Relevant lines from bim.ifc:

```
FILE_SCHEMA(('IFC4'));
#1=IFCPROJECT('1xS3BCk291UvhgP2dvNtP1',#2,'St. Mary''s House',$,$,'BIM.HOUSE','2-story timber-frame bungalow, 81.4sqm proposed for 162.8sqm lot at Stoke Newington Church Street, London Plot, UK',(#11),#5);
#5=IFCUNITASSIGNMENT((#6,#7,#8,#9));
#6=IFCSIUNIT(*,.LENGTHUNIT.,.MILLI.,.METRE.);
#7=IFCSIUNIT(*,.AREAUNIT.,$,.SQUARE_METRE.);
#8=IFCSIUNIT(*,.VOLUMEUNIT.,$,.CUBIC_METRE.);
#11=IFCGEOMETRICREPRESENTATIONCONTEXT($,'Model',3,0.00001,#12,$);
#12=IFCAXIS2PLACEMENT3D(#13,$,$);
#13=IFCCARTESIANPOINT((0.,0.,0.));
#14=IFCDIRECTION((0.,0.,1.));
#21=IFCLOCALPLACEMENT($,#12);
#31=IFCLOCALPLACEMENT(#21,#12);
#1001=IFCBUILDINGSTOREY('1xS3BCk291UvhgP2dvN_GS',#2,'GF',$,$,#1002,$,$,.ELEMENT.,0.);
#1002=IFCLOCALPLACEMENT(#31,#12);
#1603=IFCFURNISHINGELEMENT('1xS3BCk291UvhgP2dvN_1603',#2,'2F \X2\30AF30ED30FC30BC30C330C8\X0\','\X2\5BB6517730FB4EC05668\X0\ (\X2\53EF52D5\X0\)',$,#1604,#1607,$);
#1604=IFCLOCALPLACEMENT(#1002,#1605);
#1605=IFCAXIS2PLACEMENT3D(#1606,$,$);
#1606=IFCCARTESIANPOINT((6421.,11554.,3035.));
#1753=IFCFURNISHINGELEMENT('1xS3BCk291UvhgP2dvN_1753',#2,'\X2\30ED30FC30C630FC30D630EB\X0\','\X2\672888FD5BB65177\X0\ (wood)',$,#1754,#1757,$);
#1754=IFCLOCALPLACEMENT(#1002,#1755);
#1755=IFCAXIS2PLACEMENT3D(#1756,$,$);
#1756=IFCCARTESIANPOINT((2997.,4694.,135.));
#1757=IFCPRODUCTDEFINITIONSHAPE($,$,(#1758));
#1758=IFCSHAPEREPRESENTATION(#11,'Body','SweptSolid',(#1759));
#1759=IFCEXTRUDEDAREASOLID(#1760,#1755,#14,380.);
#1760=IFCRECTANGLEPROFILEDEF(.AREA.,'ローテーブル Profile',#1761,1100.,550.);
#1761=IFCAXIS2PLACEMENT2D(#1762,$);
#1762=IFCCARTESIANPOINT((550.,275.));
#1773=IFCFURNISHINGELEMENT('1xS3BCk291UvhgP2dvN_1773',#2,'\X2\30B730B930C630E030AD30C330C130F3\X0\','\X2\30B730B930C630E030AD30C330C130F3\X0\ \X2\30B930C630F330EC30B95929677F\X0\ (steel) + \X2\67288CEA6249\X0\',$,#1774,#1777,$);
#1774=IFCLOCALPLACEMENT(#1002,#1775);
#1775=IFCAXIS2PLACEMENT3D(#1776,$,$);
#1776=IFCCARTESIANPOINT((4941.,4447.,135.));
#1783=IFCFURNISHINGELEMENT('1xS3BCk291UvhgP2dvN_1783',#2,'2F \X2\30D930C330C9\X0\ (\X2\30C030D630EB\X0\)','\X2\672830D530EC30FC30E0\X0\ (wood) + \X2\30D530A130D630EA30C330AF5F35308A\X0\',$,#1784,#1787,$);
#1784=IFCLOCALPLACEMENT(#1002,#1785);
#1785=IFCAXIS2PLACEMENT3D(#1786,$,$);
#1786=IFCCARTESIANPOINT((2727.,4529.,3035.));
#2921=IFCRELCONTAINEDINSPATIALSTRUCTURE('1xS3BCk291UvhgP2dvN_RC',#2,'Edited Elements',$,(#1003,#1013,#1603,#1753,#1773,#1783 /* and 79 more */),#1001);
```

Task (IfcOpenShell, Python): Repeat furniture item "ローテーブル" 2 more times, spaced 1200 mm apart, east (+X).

```python
import numpy as np
import ifcopenshell
import ifcopenshell.api.geometry
import ifcopenshell.api.root
import ifcopenshell.util.element
import ifcopenshell.util.placement
import ifcopenshell.util.unit

model = ifcopenshell.open("bim.ifc")
unit_scale = ifcopenshell.util.unit.calculate_unit_scale(model)


def reuse_history(source, copy):
    """copy_class also copies each property set's owner history, people and application; keep the originals."""
    for rel in copy.IsDefinedBy:
        if rel.is_a("IfcRelDefinesByProperties") and (history := rel.RelatingPropertyDefinition.OwnerHistory):
            rel.RelatingPropertyDefinition.OwnerHistory = source.OwnerHistory
            ifcopenshell.util.element.remove_deep2(model, history)


source = model.by_guid("1xS3BCk291UvhgP2dvN_1753")
base = ifcopenshell.util.placement.get_local_placement(source.ObjectPlacement)
step = np.array([1.0, 0.0, 0.0]) * 1.2 / unit_scale

for i in range(1, 3):
    copy = ifcopenshell.api.root.copy_class(model, product=source)
    copy.Representation = ifcopenshell.util.element.copy_deep(
        model, source.Representation, exclude=["IfcGeometricRepresentationContext", "IfcRepresentationMap"]
    )
    reuse_history(source, copy)
    matrix = base.copy()
    matrix[:3, 3] += i * step
    print("added at", matrix[:3, 3].round(3) + 0.0)
    ifcopenshell.api.geometry.edit_object_placement(model, product=copy, matrix=matrix, is_si=False)

model.write("bim_v2.ifc")
```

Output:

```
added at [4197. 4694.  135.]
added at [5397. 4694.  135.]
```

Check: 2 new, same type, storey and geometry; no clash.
